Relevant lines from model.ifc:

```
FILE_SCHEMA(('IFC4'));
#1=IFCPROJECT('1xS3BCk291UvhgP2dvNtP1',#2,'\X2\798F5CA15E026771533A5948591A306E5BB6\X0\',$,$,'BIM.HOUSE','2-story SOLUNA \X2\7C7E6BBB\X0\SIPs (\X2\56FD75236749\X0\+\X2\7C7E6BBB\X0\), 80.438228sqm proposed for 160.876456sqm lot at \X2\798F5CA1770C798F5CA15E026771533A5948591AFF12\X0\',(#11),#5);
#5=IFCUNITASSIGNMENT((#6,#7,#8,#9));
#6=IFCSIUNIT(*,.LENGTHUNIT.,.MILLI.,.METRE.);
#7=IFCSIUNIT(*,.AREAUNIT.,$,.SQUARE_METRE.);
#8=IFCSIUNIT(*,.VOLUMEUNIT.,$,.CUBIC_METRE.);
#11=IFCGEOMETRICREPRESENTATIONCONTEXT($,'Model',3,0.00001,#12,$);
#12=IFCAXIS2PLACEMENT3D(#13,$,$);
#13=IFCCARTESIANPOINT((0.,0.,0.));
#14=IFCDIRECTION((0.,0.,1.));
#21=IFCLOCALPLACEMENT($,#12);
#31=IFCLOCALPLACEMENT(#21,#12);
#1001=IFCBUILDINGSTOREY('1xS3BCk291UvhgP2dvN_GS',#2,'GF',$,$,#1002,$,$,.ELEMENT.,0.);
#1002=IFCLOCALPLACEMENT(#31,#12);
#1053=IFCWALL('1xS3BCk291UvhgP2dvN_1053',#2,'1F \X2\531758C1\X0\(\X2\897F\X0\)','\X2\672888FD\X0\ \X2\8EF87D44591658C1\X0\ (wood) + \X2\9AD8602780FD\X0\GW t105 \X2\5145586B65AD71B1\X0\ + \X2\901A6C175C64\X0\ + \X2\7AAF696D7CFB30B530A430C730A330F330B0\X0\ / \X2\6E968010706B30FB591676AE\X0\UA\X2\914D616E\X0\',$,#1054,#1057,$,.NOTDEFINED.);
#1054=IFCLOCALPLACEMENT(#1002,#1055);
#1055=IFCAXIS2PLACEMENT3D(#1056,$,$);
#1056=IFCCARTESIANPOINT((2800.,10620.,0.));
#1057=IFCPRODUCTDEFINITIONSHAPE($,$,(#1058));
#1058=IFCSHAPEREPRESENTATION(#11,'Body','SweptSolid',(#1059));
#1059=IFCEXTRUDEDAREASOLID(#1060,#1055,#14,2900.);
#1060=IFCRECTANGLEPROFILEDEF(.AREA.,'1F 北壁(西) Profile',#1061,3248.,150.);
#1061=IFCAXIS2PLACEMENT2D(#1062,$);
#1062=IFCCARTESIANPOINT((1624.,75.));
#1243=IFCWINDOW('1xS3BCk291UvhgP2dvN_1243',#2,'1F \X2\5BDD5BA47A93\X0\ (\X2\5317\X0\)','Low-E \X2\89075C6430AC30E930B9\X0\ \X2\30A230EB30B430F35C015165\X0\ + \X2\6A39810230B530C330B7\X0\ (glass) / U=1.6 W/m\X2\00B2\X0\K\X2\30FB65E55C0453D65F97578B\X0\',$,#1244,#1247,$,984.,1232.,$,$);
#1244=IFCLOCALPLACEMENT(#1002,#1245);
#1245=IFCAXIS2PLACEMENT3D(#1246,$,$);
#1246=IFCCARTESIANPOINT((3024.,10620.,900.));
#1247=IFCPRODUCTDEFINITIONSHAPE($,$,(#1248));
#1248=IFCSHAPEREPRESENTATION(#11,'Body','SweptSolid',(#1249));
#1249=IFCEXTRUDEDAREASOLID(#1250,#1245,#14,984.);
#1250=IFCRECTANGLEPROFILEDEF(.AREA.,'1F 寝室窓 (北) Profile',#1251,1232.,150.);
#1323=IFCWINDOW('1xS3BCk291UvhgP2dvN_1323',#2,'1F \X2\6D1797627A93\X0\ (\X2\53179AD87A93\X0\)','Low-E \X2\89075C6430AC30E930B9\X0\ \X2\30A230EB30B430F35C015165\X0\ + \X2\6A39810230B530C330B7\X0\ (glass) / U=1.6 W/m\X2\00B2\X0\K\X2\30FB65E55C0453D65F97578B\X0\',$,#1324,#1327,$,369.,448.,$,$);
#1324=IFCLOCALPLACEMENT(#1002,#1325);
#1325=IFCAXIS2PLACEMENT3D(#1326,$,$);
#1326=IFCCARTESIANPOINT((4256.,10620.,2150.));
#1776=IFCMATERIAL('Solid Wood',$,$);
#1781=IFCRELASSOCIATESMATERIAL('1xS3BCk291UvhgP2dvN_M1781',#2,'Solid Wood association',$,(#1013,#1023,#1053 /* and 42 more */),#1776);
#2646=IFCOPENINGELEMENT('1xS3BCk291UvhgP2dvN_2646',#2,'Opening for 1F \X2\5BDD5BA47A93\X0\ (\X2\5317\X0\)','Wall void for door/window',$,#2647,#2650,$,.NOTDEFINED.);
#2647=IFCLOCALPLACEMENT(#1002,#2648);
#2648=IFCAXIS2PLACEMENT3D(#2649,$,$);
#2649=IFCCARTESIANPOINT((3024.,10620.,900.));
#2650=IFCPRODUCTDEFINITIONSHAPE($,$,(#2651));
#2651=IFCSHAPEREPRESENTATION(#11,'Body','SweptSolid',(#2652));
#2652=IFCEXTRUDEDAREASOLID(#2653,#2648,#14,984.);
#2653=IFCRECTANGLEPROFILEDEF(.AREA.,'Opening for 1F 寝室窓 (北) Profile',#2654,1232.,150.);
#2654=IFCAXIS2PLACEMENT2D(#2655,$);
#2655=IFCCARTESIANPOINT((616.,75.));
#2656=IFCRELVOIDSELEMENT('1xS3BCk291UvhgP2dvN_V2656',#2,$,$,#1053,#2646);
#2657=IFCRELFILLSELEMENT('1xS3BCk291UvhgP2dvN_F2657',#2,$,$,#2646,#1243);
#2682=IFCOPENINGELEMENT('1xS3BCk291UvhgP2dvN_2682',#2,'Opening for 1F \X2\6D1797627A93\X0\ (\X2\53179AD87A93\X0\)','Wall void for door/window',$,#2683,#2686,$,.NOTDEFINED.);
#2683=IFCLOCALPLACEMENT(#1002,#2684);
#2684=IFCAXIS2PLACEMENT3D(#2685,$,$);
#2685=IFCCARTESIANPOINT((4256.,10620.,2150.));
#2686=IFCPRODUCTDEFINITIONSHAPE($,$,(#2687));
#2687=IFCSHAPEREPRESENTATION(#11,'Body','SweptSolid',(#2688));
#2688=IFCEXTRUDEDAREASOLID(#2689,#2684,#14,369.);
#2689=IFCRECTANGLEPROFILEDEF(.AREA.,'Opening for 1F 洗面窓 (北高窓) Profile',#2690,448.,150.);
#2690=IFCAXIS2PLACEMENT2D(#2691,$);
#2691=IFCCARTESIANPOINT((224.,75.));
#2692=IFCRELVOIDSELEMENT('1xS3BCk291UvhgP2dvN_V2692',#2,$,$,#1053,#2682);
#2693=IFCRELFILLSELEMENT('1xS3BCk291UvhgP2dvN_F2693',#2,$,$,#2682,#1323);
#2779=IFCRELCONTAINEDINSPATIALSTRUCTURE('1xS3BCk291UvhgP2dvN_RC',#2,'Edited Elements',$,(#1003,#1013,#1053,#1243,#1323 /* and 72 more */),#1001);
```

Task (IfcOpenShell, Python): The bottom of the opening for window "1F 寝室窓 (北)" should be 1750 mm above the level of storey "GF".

```python
import numpy as np
import ifcopenshell
import ifcopenshell.api.geometry
import ifcopenshell.geom
import ifcopenshell.util.element
import ifcopenshell.util.placement
import ifcopenshell.util.shape
import ifcopenshell.util.unit

model = ifcopenshell.open("model.ifc")
unit_scale = ifcopenshell.util.unit.calculate_unit_scale(model)

window = model.by_guid("1xS3BCk291UvhgP2dvN_1243")
opening = window.FillsVoids[0].RelatingOpeningElement
storey = ifcopenshell.util.element.get_container(window, ifc_class="IfcBuildingStorey")
level = ifcopenshell.util.placement.get_local_placement(storey.ObjectPlacement)[2, 3]

# The opening's origin need not be at the sill, so measure its lowest point.
shape = ifcopenshell.geom.create_shape(ifcopenshell.geom.settings(), opening)
bottom = ifcopenshell.util.shape.get_shape_bottom_elevation(shape, shape.geometry) / unit_scale
dz = level + 1.75 / unit_scale - bottom

shift = np.array([0.0, 0.0, dz])
# The window is not placed relative to its opening, so move both.
for product in (opening, window):
    matrix = ifcopenshell.util.placement.get_local_placement(product.ObjectPlacement)
    matrix[:3, 3] += shift
    ifcopenshell.api.geometry.edit_object_placement(model, product=product, matrix=matrix, is_si=False)

print(f"moved by {dz * unit_scale:+.3f} m")

model.write("model_rev.ifc")
```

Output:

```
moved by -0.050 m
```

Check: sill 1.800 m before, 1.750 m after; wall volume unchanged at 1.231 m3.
